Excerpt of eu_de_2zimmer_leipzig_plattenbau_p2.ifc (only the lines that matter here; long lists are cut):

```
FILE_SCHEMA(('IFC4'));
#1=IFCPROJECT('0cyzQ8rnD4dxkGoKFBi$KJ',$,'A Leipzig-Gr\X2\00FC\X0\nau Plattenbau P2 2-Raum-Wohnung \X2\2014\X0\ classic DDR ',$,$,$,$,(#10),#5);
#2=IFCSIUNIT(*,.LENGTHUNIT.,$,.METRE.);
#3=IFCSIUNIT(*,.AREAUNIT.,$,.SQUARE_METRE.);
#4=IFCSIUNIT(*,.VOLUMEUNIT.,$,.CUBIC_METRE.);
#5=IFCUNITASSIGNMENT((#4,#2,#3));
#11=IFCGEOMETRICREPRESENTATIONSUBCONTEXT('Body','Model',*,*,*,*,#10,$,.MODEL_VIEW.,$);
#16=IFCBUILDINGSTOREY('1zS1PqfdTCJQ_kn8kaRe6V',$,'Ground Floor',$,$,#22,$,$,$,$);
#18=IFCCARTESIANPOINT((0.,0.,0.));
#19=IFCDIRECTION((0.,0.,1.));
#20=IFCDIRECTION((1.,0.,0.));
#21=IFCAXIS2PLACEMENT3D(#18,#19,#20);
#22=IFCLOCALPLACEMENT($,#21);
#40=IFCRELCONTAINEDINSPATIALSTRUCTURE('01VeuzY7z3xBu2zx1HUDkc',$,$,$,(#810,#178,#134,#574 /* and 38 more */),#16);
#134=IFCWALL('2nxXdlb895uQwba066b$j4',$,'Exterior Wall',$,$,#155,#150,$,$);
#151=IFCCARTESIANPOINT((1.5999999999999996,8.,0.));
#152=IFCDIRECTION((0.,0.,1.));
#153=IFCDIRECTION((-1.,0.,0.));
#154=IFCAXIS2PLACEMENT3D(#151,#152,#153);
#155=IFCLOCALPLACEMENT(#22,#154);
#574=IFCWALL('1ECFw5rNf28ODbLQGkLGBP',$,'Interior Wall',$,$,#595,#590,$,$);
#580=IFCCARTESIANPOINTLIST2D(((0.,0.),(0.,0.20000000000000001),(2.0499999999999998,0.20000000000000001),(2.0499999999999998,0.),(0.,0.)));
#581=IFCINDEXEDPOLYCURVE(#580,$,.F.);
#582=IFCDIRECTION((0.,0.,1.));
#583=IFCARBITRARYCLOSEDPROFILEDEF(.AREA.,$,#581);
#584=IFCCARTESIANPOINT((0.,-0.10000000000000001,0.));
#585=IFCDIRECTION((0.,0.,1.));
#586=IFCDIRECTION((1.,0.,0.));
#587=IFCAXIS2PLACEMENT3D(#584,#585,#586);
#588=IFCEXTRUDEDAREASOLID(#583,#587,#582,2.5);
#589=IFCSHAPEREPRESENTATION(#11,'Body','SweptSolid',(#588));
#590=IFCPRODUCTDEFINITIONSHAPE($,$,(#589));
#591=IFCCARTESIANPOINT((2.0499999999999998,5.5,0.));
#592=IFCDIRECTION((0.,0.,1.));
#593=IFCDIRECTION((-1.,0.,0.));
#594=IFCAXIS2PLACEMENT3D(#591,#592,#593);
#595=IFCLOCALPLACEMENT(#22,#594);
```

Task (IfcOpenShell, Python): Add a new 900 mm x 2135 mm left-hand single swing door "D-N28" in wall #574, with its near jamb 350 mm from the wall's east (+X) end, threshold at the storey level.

```python
import numpy as np
import ifcopenshell
import ifcopenshell.api.feature
import ifcopenshell.api.geometry
import ifcopenshell.api.root
import ifcopenshell.api.spatial
import ifcopenshell.geom
import ifcopenshell.util.element
import ifcopenshell.util.placement
import ifcopenshell.util.representation
import ifcopenshell.util.shape
import ifcopenshell.util.unit

model = ifcopenshell.open("eu_de_2zimmer_leipzig_plattenbau_p2.ifc")
unit_scale = ifcopenshell.util.unit.calculate_unit_scale(model)
settings = ifcopenshell.geom.settings()


def volume(element):
    """Net volume in cubic metres, openings subtracted."""
    shape = ifcopenshell.geom.create_shape(settings, element)
    return ifcopenshell.util.shape.get_volume(shape.geometry)


wall = model.by_guid("1ECFw5rNf28ODbLQGkLGBP")
storey = ifcopenshell.util.element.get_container(wall, ifc_class="IfcBuildingStorey")
context = ifcopenshell.util.representation.get_context(model, "Model", "Body", "MODEL_VIEW")
before = volume(wall)

width, height, from_end, sill = 0.9, 2.135, 0.35, 0.0  # metres

# The wall runs along its own X axis, and the end named is its -X end.
wall_shape = ifcopenshell.geom.create_shape(settings, wall)
x, y, z = ifcopenshell.util.shape.get_vertices(wall_shape.geometry).T
start = x.min() + from_end
face, thickness = float(y.min()), float(y.max() - y.min())
wall_matrix = ifcopenshell.util.placement.get_local_placement(wall.ObjectPlacement)
level = ifcopenshell.util.placement.get_local_placement(storey.ObjectPlacement)[2, 3]


def in_wall(x, y):
    """Placement at x, y metres in the wall's axes, at sill height."""
    matrix = wall_matrix.copy()
    matrix[:, 3] = wall_matrix @ np.array([x / unit_scale, y / unit_scale, 0.0, 1.0])
    matrix[2, 3] = level + sill / unit_scale
    return matrix


# Opening: a box that overshoots both wall faces by 50 mm.
opening = ifcopenshell.api.root.create_entity(model, ifc_class="IfcOpeningElement", predefined_type="OPENING")
box = ifcopenshell.api.geometry.add_wall_representation(
    model, context=context, length=width, height=height, thickness=thickness + 0.1
)
ifcopenshell.api.geometry.assign_representation(model, product=opening, representation=box)
ifcopenshell.api.geometry.edit_object_placement(model, product=opening, matrix=in_wall(start, face - 0.05), is_si=False)
ifcopenshell.api.feature.add_feature(model, feature=opening, element=wall)

door = ifcopenshell.api.root.create_entity(model, ifc_class="IfcDoor", name="D-N28", predefined_type="DOOR")
door.OverallWidth, door.OverallHeight = width / unit_scale, height / unit_scale
door.OperationType = "SINGLE_SWING_LEFT"
body = ifcopenshell.api.geometry.add_door_representation(
    model,
    context=context,
    overall_width=door.OverallWidth,
    overall_height=door.OverallHeight,
    operation_type="SINGLE_SWING_LEFT",
    lining_properties={"LiningDepth": thickness / unit_scale, "ThresholdDepth": thickness / unit_scale},
)
ifcopenshell.api.geometry.assign_representation(model, product=door, representation=body)
ifcopenshell.api.spatial.assign_container(model, products=[door], relating_structure=storey)
ifcopenshell.api.feature.add_filling(model, opening=opening, element=door)

# The lining spans the wall, so the door starts at the wall face.
ifcopenshell.api.geometry.edit_object_placement(model, product=door, matrix=in_wall(start, face), is_si=False)

after = volume(wall)

print(f"wall volume {before:.3f} -> {after:.3f} m3")

model.write("eu_de_2zimmer_leipzig_plattenbau_p2_edited.ifc")
```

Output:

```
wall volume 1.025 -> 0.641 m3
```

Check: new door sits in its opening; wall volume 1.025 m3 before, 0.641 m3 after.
